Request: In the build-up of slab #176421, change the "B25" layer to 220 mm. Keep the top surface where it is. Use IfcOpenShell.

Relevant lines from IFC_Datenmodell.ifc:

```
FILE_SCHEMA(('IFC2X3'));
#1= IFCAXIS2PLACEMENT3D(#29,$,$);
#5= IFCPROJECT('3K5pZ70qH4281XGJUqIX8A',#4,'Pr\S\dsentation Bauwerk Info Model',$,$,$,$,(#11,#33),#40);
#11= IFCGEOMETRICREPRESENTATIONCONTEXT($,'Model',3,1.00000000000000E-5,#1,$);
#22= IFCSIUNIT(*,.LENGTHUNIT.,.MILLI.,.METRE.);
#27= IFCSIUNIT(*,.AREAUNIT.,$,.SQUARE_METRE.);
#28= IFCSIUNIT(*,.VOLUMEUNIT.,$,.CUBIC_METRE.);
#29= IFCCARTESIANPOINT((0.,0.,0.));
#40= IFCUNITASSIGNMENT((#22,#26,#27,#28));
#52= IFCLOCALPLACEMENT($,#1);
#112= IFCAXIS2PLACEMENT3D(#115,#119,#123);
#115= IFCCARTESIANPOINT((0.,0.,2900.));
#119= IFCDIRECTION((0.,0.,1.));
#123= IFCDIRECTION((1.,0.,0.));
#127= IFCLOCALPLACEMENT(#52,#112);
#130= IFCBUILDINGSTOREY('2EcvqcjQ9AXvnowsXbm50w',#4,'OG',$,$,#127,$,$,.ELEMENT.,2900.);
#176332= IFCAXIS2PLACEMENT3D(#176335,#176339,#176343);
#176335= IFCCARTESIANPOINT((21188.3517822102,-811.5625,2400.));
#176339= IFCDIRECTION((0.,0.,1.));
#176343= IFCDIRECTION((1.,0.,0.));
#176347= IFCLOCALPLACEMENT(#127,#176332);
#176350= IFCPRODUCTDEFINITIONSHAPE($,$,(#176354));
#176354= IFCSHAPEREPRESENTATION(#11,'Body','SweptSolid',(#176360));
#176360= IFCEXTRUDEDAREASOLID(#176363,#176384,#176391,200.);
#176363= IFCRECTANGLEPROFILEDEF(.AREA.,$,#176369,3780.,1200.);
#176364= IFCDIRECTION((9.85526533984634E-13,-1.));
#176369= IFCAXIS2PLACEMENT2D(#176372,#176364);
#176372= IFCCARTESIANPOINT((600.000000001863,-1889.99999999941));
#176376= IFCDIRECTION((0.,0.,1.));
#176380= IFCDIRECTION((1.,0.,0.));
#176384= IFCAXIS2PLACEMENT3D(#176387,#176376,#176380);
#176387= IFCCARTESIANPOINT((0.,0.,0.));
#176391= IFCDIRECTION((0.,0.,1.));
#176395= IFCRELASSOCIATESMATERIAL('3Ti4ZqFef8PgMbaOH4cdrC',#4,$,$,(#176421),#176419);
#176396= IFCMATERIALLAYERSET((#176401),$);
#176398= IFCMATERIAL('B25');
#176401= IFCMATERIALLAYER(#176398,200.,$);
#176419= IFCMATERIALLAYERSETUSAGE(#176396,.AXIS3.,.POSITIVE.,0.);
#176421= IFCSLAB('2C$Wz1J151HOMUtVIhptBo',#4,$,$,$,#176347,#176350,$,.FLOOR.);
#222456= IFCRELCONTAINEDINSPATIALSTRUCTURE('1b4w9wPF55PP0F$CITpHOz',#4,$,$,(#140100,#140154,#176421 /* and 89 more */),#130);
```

```python
import ifcopenshell
import ifcopenshell.util.element

model = ifcopenshell.open("IFC_Datenmodell.ifc")

layer_set = model.by_id(176396)
layer = next(l for l in layer_set.MaterialLayers if l.Material and l.Material.Name == "B25")
change = 220.0 - layer.LayerThickness
layer.LayerThickness += change

# Geometry does not follow the layer set by itself.
slabs = [e for e in ifcopenshell.util.element.get_elements_by_material(model, layer_set) if e.is_a("IfcSlab")]
for slab in sorted(slabs, key=lambda e: e.id()):
    body = next(r for r in slab.Representation.Representations if r.RepresentationIdentifier == "Body")
    solid = body.Items[0]
    old_depth = solid.Depth
    solid.Depth += change
    # Extruded upwards: lower the start of the extrusion so the top stays.
    x, y, z = solid.Position.Location.Coordinates
    solid.Position.Location = model.createIfcCartesianPoint((x, y, z - change))
    print(slab.id(), f"{old_depth:g} -> {solid.Depth:g}")

# The layers are counted up from the underside, which has moved.
for usage in {ifcopenshell.util.element.get_material(slab) for slab in slabs}:
    usage.OffsetFromReferenceLine -= change

model.write("IFC_Datenmodell_updated.ifc")
```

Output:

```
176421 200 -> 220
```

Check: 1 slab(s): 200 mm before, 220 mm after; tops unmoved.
